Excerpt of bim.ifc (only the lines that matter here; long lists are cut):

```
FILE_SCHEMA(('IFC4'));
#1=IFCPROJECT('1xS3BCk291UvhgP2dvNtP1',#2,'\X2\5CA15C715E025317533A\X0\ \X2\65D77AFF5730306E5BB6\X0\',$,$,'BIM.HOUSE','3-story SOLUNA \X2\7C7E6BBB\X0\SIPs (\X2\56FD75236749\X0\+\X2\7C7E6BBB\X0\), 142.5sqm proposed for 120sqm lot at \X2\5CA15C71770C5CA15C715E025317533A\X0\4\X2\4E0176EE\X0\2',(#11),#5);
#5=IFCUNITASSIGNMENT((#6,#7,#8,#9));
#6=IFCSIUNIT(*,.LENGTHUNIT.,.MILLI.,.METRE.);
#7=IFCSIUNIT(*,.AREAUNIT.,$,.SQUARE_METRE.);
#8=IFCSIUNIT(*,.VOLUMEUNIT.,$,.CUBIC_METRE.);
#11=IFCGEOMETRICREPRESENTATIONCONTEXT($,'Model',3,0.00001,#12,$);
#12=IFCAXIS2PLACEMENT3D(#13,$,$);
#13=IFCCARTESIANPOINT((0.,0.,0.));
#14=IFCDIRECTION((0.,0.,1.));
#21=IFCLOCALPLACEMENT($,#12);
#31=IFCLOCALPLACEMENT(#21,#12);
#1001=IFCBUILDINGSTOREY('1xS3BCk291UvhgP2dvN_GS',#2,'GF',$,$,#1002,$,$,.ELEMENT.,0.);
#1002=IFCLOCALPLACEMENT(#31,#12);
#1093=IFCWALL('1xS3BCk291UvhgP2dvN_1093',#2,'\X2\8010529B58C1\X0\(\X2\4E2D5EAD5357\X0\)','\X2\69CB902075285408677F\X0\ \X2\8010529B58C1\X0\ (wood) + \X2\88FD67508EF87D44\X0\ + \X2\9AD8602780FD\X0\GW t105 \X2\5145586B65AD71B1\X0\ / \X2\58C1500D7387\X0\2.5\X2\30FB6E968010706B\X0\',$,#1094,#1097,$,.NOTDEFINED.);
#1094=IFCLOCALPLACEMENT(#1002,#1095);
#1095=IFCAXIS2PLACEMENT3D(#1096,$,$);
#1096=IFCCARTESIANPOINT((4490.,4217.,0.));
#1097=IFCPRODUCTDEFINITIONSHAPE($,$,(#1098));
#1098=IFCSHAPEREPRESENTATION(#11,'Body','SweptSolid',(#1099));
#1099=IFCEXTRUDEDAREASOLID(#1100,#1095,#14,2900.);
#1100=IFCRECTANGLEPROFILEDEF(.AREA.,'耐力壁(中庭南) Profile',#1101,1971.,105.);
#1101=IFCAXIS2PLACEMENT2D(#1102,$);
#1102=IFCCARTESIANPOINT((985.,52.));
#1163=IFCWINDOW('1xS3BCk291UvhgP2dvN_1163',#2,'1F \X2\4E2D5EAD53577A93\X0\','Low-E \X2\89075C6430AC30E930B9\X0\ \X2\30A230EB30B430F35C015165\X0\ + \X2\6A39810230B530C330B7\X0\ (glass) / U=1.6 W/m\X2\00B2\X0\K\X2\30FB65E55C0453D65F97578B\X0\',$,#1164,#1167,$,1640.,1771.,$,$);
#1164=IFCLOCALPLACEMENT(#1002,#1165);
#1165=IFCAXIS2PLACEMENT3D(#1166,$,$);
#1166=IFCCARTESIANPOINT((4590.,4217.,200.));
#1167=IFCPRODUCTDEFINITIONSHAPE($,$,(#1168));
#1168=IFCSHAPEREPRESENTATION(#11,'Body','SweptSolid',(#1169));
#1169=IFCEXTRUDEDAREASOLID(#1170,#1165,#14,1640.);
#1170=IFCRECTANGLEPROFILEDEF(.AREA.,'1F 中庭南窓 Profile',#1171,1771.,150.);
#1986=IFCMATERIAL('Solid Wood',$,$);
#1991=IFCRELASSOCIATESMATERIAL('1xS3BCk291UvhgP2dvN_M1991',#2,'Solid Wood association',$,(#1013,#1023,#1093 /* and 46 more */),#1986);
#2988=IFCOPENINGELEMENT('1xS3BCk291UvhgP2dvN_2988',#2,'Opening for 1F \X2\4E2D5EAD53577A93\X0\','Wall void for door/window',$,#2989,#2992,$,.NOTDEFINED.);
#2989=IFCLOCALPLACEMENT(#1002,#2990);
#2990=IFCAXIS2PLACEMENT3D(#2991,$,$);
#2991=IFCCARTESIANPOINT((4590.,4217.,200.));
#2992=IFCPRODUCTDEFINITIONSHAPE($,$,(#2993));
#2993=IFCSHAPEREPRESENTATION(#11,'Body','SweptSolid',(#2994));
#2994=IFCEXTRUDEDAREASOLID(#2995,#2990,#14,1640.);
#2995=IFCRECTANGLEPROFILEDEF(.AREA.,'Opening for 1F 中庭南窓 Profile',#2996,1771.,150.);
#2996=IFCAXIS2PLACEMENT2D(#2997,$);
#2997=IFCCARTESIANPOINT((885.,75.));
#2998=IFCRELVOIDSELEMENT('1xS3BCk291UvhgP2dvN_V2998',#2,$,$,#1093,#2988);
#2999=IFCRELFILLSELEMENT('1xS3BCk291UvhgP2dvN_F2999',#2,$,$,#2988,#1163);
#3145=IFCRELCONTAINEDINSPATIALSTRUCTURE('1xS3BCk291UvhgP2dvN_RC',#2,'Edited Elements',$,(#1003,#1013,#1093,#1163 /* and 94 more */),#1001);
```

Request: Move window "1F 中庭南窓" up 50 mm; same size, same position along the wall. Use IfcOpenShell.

```python
import numpy as np
import ifcopenshell
import ifcopenshell.api.geometry
import ifcopenshell.util.placement
import ifcopenshell.util.unit

model = ifcopenshell.open("bim.ifc")
unit_scale = ifcopenshell.util.unit.calculate_unit_scale(model)

window = model.by_guid("1xS3BCk291UvhgP2dvN_1163")
opening = window.FillsVoids[0].RelatingOpeningElement
dz = 0.05 / unit_scale

shift = np.array([0.0, 0.0, dz])
# The window is not placed relative to its opening, so move both.
for product in (opening, window):
    matrix = ifcopenshell.util.placement.get_local_placement(product.ObjectPlacement)
    matrix[:3, 3] += shift
    ifcopenshell.api.geometry.edit_object_placement(model, product=product, matrix=matrix, is_si=False)

print(f"moved by {dz * unit_scale:+.3f} m")

model.write("bim_v2.ifc")
```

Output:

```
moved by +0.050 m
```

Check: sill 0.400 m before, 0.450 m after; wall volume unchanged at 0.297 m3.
